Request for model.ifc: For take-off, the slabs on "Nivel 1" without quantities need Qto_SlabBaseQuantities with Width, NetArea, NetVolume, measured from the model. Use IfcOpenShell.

First a look at what the model holds.

```python
import ifcopenshell
import ifcopenshell.util.element
import ifcopenshell.util.unit

model = ifcopenshell.open("model.ifc")
print(model.schema)
for unit_type in ("LENGTHUNIT", "AREAUNIT", "VOLUMEUNIT"):
    print(unit_type, ifcopenshell.util.unit.calculate_unit_scale(model, unit_type))
storey = next(s for s in model.by_type("IfcBuildingStorey") if s.Name == "Nivel 1")
slabs = [e for e in ifcopenshell.util.element.get_decomposition(storey) if e.is_a("IfcSlab")]
for e in sorted(slabs, key=lambda e: e.id()):
    print(e.id(), e.is_a(), e.Name, list(ifcopenshell.util.element.get_psets(e, qtos_only=True)), sep=" | ")
```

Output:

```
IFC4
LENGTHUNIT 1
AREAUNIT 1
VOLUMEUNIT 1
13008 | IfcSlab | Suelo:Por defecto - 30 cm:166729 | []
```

```python
import ifcopenshell
import ifcopenshell.api.pset
import ifcopenshell.geom
import ifcopenshell.util.element
import ifcopenshell.util.shape
import ifcopenshell.util.unit

model = ifcopenshell.open("model.ifc")
unit_scale = ifcopenshell.util.unit.calculate_unit_scale(model)
area_scale = ifcopenshell.util.unit.calculate_unit_scale(model, "AREAUNIT")
volume_scale = ifcopenshell.util.unit.calculate_unit_scale(model, "VOLUMEUNIT")
settings = ifcopenshell.geom.settings()

storey = next(s for s in model.by_type("IfcBuildingStorey") if s.Name == "Nivel 1")
slabs = [e for e in ifcopenshell.util.element.get_decomposition(storey) if e.is_a("IfcSlab")]

for e in sorted(slabs, key=lambda e: e.id()):
    if ifcopenshell.util.element.get_psets(e, qtos_only=True, should_inherit=False):
        continue
    # Geometry comes back in metres, in the element's own axes.
    shape = ifcopenshell.geom.create_shape(settings, e)
    values = {
        "Width": ifcopenshell.util.shape.get_z(shape.geometry) / unit_scale,
        "NetArea": ifcopenshell.util.shape.get_footprint_area(shape.geometry) / area_scale,
        "NetVolume": ifcopenshell.util.shape.get_volume(shape.geometry) / volume_scale,
    }
    qto = ifcopenshell.api.pset.add_qto(model, product=e, name="Qto_SlabBaseQuantities")
    ifcopenshell.api.pset.edit_qto(model, qto=qto, properties=values)
    print(e.id(), {k: round(v, 3) for k, v in values.items()})

model.write("model_v2.ifc")
```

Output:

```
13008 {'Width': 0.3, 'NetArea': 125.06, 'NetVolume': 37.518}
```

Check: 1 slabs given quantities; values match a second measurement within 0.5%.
